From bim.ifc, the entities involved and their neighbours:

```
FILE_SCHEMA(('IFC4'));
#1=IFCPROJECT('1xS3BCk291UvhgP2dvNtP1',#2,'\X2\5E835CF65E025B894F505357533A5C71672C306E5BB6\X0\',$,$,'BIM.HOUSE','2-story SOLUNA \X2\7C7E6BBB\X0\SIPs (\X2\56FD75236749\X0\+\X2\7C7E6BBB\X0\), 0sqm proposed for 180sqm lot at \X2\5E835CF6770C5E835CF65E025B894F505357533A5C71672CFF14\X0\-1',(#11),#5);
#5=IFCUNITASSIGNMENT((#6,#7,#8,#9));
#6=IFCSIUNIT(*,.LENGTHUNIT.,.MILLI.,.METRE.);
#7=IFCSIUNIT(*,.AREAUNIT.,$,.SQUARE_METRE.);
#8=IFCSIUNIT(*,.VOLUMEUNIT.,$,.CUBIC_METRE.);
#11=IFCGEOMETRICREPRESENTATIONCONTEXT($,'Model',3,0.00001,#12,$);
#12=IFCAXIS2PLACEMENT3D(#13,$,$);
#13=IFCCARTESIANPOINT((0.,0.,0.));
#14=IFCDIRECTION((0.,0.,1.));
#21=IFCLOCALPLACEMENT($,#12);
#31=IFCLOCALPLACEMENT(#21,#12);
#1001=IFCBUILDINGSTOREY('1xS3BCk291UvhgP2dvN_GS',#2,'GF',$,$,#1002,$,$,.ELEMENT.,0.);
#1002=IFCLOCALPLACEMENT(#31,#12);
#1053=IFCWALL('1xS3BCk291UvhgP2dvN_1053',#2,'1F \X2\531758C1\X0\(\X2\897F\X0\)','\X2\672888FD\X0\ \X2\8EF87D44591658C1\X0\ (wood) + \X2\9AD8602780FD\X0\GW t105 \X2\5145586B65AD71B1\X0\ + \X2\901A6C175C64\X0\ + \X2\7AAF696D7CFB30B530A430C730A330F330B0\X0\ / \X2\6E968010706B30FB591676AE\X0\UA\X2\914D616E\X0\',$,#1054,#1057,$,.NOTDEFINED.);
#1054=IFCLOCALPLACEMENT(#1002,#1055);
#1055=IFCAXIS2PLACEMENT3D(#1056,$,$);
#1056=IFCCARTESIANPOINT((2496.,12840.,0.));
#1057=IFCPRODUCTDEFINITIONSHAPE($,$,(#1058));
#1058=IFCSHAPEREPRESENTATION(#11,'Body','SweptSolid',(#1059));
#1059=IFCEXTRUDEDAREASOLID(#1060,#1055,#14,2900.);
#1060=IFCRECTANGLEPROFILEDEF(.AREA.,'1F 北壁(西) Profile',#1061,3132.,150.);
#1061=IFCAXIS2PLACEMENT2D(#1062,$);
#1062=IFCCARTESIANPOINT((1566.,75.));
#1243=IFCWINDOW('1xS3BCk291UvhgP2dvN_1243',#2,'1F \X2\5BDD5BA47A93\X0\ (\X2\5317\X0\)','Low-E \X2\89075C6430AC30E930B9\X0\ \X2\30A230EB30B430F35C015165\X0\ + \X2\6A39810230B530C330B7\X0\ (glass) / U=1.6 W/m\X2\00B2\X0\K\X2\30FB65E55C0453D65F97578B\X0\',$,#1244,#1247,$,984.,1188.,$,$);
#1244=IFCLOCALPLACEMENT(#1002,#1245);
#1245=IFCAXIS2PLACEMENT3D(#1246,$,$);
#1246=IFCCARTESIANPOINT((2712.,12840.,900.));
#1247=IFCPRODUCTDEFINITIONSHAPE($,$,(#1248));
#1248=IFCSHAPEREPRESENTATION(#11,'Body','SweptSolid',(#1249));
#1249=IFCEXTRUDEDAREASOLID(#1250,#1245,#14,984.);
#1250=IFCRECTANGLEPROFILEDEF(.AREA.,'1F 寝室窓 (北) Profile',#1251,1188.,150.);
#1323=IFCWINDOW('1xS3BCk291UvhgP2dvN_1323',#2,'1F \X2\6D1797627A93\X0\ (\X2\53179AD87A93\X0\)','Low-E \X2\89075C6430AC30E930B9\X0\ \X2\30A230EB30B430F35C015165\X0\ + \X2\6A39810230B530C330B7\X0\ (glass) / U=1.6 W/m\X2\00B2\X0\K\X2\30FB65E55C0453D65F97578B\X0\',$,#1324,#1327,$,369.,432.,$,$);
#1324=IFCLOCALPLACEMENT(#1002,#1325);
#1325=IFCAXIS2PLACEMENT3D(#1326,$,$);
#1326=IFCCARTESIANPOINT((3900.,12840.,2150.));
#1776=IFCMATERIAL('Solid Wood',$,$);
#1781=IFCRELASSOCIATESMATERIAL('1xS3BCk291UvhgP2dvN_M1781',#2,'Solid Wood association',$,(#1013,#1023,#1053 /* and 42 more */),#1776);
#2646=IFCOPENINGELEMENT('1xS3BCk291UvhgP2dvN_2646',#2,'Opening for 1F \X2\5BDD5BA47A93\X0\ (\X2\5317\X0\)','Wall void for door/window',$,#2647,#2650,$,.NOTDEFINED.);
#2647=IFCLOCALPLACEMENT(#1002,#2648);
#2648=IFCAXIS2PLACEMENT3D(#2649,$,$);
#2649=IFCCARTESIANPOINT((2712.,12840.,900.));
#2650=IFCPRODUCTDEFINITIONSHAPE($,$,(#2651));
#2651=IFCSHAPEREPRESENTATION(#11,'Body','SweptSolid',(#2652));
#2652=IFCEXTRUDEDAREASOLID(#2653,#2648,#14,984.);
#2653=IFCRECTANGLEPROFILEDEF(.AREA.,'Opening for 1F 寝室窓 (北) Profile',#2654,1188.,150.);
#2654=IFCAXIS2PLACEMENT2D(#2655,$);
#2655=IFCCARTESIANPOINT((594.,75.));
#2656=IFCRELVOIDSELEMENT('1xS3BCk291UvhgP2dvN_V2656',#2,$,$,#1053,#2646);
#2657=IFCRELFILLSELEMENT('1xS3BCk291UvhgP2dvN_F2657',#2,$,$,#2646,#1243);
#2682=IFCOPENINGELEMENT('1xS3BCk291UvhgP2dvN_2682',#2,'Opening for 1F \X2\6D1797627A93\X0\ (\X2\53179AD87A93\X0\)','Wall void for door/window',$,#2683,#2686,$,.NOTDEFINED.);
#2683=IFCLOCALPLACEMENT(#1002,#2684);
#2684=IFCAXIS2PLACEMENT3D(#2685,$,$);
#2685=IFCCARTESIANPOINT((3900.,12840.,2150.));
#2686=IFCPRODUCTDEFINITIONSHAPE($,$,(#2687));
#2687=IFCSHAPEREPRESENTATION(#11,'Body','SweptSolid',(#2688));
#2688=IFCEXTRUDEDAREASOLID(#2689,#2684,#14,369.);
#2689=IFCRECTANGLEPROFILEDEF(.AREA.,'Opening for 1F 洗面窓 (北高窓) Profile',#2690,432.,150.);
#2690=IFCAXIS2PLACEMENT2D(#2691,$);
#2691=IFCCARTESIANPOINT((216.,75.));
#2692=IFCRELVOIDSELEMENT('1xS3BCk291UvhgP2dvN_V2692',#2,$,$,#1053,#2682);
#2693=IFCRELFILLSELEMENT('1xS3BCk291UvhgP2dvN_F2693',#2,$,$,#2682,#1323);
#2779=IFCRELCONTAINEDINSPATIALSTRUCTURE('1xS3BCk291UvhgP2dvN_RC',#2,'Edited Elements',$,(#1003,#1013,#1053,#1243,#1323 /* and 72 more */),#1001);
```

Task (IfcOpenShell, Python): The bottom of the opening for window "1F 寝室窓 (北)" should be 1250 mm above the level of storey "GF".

```python
import numpy as np
import ifcopenshell
import ifcopenshell.api.geometry
import ifcopenshell.geom
import ifcopenshell.util.element
import ifcopenshell.util.placement
import ifcopenshell.util.shape
import ifcopenshell.util.unit

model = ifcopenshell.open("bim.ifc")
unit_scale = ifcopenshell.util.unit.calculate_unit_scale(model)

window = model.by_guid("1xS3BCk291UvhgP2dvN_1243")
opening = window.FillsVoids[0].RelatingOpeningElement
storey = ifcopenshell.util.element.get_container(window, ifc_class="IfcBuildingStorey")
level = ifcopenshell.util.placement.get_local_placement(storey.ObjectPlacement)[2, 3]

# The opening's origin need not be at the sill, so measure its lowest point.
shape = ifcopenshell.geom.create_shape(ifcopenshell.geom.settings(), opening)
bottom = ifcopenshell.util.shape.get_shape_bottom_elevation(shape, shape.geometry) / unit_scale
dz = level + 1250.0 - bottom

shift = np.array([0.0, 0.0, dz])
# The window is not placed relative to its opening, so move both.
for product in (opening, window):
    matrix = ifcopenshell.util.placement.get_local_placement(product.ObjectPlacement)
    matrix[:3, 3] += shift
    ifcopenshell.api.geometry.edit_object_placement(model, product=product, matrix=matrix, is_si=False)

print(f"moved by {dz * unit_scale:+.3f} m")

model.write("bim_updated.ifc")
```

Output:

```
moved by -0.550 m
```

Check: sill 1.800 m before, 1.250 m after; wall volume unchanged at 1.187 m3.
